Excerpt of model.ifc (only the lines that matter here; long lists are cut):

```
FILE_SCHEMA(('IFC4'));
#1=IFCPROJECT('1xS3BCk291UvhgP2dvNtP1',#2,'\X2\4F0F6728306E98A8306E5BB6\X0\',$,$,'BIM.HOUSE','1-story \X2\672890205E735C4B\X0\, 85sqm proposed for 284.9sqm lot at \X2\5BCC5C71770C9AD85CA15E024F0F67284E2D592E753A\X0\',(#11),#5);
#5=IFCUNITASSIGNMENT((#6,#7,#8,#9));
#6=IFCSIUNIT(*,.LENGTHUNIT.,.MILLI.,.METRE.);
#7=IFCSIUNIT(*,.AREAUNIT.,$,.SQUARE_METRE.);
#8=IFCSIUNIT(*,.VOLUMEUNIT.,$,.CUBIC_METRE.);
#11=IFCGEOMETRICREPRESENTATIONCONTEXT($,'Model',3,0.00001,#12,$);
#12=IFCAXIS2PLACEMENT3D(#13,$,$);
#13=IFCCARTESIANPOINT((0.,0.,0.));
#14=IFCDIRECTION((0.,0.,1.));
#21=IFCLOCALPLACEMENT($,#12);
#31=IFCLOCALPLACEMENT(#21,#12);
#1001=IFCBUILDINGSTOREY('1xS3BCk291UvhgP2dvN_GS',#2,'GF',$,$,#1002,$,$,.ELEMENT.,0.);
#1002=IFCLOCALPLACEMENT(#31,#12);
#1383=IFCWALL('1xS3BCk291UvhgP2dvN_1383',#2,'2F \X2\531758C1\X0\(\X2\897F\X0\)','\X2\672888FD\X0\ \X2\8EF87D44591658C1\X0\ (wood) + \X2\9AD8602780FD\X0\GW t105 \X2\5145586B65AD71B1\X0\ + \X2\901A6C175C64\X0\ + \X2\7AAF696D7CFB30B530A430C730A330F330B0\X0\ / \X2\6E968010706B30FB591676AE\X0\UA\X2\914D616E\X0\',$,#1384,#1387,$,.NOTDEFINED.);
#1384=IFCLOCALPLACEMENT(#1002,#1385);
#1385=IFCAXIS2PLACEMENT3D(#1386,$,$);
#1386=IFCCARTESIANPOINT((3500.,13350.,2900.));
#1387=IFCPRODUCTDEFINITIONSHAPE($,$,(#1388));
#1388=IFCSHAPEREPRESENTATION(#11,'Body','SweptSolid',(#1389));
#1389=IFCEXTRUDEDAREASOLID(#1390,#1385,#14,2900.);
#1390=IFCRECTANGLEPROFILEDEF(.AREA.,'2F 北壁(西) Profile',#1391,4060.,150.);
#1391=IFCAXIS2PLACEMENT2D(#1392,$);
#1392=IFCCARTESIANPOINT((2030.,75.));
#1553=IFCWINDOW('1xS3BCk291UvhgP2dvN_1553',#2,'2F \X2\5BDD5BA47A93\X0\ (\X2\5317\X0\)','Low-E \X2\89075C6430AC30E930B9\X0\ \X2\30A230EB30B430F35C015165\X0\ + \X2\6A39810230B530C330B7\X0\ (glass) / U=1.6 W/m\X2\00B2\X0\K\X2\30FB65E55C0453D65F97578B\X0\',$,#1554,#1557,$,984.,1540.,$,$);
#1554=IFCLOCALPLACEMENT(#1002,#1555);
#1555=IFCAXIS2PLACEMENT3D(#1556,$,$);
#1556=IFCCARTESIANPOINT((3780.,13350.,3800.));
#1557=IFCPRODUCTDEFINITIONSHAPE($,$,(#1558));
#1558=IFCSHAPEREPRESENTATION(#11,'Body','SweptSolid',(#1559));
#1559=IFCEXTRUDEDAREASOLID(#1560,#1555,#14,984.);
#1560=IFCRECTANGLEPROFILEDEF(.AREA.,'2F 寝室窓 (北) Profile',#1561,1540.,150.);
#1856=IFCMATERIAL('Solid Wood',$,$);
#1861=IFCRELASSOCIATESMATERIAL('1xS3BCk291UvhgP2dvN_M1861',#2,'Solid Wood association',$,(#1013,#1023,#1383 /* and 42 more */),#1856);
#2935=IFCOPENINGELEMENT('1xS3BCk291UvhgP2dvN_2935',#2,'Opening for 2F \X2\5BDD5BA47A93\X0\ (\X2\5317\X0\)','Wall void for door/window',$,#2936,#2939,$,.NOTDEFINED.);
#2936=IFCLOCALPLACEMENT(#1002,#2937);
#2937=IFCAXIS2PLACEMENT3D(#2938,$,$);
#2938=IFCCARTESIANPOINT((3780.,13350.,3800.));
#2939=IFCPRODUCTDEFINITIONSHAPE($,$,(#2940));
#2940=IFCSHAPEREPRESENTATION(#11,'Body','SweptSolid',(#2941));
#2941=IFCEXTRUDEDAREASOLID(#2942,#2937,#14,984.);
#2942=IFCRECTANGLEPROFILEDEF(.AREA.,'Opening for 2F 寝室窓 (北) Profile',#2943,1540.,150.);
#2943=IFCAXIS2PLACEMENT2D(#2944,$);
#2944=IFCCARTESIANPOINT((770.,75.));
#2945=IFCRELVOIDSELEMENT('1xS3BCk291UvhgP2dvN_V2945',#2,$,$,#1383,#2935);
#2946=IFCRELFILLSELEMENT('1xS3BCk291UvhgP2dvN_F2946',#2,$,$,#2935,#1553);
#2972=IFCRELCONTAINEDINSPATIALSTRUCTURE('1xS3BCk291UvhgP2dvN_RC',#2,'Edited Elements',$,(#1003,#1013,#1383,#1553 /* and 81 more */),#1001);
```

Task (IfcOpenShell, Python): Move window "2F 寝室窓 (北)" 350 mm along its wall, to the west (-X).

```python
import ifcopenshell
import ifcopenshell.api.geometry
import ifcopenshell.util.placement

model = ifcopenshell.open("model.ifc")

window = model.by_guid("1xS3BCk291UvhgP2dvN_1553")
opening = window.FillsVoids[0].RelatingOpeningElement
wall = opening.VoidsElements[0].RelatingBuildingElement

wall_matrix = ifcopenshell.util.placement.get_local_placement(wall.ObjectPlacement)
shift = wall_matrix[:3, 0] * -350.0
before = ifcopenshell.util.placement.get_local_placement(window.ObjectPlacement)[:3, 3].copy()

# The window is not placed relative to its opening, so move both.
for product in (opening, window):
    matrix = ifcopenshell.util.placement.get_local_placement(product.ObjectPlacement)
    matrix[:3, 3] += shift
    ifcopenshell.api.geometry.edit_object_placement(model, product=product, matrix=matrix, is_si=False)

after = ifcopenshell.util.placement.get_local_placement(window.ObjectPlacement)[:3, 3]
print("window moved by", (after - before).round(3) + 0.0)

model.write("model_edited.ifc")
```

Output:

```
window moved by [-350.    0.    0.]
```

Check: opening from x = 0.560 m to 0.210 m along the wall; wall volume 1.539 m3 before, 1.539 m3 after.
